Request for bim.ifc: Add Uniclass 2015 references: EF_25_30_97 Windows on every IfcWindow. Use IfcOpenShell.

First a look at what the model holds.

```python
import ifcopenshell

model = ifcopenshell.open("bim.ifc")
print(model.schema)
print("classifications:", [c.Name for c in model.by_type("IfcClassification")])
for ifc_class in ("IfcDoor", "IfcRoof", "IfcStair", "IfcWall", "IfcWindow"):
    print(ifc_class, len(model.by_type(ifc_class)))
```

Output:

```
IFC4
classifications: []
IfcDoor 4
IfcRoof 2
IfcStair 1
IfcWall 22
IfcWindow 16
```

```python
import ifcopenshell
import ifcopenshell.api.classification

model = ifcopenshell.open("bim.ifc")

system = ifcopenshell.api.classification.add_classification(model, classification="Uniclass 2015")

codes = {
    "IfcWindow": ("EF_25_30_97", "Windows"),
}
for ifc_class, (code, name) in codes.items():
    products = model.by_type(ifc_class)
    ifcopenshell.api.classification.add_reference(
        model, products=products, classification=system, identification=code, name=name
    )
    print(code, len(products))

model.write("bim-out.ifc")
```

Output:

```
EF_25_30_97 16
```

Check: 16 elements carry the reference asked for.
